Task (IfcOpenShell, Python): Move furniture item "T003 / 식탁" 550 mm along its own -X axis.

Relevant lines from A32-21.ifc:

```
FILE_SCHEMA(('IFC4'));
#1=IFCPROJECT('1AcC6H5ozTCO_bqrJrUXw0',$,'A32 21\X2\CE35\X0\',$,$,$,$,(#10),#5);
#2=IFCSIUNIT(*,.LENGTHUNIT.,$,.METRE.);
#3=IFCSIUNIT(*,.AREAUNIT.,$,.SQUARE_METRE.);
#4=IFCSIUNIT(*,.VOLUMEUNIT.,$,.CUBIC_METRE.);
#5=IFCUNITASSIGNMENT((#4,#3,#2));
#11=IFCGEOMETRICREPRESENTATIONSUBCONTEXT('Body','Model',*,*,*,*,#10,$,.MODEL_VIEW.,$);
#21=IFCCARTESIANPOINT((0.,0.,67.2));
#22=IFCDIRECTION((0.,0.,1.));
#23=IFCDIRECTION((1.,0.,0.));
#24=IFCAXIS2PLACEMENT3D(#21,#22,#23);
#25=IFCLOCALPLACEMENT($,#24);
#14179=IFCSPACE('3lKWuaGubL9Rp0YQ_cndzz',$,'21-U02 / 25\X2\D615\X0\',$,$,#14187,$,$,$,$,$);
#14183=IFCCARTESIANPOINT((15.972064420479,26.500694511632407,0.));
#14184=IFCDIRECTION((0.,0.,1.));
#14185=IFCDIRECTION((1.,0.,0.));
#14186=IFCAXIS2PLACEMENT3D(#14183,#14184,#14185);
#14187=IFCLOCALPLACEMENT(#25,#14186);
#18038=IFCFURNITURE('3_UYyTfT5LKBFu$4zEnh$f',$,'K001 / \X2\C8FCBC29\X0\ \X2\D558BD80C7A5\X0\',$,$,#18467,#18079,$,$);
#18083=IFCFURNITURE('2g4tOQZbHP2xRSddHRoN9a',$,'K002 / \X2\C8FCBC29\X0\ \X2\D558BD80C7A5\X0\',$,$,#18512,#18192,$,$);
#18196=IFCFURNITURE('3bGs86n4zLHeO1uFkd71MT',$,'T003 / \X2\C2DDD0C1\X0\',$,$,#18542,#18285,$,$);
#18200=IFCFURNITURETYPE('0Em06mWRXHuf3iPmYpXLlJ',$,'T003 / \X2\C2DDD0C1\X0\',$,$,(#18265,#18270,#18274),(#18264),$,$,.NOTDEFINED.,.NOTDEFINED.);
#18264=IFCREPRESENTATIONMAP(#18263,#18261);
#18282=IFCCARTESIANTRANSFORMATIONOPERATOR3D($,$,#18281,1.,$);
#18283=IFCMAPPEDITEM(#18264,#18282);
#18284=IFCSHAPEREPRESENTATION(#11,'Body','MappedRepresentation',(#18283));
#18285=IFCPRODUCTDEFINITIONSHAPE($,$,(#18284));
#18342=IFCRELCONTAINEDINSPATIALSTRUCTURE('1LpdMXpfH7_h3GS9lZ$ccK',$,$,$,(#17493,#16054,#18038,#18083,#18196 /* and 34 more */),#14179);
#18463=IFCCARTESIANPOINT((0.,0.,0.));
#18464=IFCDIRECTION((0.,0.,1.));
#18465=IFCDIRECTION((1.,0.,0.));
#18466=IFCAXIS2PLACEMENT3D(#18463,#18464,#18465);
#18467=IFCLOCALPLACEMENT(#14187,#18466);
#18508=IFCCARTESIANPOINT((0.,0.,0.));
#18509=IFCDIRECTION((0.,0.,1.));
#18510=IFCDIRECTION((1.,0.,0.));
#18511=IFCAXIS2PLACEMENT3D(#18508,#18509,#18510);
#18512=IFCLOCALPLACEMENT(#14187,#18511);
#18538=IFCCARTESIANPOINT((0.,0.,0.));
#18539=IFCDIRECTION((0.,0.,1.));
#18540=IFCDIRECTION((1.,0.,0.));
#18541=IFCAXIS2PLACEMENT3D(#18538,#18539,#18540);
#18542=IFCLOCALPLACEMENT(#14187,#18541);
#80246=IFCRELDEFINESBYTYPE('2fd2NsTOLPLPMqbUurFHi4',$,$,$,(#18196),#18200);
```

```python
import ifcopenshell
import ifcopenshell.api.geometry
import ifcopenshell.util.placement
import ifcopenshell.util.unit

model = ifcopenshell.open("A32-21.ifc")
unit_scale = ifcopenshell.util.unit.calculate_unit_scale(model)

item = model.by_id(18196)
matrix = ifcopenshell.util.placement.get_local_placement(item.ObjectPlacement)
matrix[:3, 3] -= matrix[:3, 0] * 0.55 / unit_scale
ifcopenshell.api.geometry.edit_object_placement(model, product=item, matrix=matrix, is_si=False)

print(ifcopenshell.util.placement.get_local_placement(item.ObjectPlacement).round(3) + 0.0)

model.write("A32-21_rev.ifc")
```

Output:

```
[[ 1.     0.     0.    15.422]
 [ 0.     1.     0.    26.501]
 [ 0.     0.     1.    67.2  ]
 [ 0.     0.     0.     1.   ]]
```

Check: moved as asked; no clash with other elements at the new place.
